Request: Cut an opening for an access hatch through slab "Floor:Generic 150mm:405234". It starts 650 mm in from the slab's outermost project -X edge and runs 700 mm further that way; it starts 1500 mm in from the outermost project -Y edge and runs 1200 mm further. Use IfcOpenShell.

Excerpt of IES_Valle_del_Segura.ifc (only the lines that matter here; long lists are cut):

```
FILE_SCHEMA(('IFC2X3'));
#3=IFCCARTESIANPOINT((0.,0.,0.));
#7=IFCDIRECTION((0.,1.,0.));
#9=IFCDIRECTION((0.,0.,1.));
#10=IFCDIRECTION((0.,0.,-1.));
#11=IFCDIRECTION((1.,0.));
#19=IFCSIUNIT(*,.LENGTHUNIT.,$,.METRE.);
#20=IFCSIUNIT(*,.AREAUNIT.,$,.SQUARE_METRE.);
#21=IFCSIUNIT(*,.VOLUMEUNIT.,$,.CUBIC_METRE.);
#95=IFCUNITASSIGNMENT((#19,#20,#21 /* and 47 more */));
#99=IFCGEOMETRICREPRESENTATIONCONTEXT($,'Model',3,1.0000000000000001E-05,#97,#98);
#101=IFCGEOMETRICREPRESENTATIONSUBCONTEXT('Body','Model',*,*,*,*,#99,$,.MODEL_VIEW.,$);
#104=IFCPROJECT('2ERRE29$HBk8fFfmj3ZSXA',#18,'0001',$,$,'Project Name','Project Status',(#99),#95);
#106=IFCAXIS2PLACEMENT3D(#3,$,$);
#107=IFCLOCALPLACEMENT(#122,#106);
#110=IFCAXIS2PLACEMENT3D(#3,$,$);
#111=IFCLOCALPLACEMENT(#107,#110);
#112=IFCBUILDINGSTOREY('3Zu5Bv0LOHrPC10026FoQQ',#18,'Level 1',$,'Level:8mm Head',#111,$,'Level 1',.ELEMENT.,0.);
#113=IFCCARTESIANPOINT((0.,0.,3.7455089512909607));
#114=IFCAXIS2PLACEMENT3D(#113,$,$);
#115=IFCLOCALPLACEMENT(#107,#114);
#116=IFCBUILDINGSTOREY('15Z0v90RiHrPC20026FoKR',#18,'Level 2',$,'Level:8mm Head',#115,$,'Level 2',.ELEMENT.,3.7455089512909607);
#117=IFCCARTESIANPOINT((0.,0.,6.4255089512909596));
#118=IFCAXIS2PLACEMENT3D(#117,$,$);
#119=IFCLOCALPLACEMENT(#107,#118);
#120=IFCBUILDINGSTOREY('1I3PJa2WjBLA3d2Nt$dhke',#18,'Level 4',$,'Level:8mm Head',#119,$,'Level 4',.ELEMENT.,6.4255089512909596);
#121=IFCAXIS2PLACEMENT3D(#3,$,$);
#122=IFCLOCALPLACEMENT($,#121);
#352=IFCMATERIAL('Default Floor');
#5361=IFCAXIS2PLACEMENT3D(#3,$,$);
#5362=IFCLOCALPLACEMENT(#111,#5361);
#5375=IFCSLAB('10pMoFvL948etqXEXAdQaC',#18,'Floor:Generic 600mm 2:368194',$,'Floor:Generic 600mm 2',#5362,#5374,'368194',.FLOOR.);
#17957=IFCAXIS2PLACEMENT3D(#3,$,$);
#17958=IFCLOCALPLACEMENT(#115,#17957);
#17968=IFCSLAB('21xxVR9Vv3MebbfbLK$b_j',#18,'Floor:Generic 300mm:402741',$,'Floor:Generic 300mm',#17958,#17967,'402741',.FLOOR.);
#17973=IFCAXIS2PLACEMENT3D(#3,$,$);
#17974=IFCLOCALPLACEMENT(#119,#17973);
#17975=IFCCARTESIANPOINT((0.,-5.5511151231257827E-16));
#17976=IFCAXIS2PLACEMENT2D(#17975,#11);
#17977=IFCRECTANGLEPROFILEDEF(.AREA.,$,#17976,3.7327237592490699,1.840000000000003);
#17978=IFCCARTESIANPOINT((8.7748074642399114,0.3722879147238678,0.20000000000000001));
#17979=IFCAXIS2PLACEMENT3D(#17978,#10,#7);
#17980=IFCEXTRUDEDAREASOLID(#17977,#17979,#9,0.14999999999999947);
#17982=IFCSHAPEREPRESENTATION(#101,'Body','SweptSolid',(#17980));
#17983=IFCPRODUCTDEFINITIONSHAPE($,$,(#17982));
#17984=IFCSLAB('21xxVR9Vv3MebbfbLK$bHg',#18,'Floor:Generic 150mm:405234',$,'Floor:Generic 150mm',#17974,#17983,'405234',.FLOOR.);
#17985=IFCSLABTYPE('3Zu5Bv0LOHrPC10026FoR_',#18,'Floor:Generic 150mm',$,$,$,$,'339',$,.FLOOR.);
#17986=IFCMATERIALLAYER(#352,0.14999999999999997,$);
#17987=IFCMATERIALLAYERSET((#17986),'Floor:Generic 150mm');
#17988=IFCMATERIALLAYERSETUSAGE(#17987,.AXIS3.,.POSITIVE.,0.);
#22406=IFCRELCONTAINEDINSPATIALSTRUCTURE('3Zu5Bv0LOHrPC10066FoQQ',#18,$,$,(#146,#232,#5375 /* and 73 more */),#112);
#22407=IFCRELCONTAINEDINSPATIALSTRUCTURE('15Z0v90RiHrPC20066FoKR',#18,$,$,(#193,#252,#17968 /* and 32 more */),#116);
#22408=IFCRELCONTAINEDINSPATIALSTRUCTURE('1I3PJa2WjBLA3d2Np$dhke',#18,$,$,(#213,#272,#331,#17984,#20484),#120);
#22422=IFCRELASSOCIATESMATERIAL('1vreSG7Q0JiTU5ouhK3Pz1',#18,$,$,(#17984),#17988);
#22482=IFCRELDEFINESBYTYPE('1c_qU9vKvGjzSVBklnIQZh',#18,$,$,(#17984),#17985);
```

```python
import numpy as np
import ifcopenshell
import ifcopenshell.api.feature
import ifcopenshell.api.geometry
import ifcopenshell.api.root
import ifcopenshell.geom
import ifcopenshell.util.placement
import ifcopenshell.util.representation
import ifcopenshell.util.shape
import ifcopenshell.util.unit

model = ifcopenshell.open("IES_Valle_del_Segura.ifc")
unit_scale = ifcopenshell.util.unit.calculate_unit_scale(model)
settings = ifcopenshell.geom.settings()


def volume(element):
    """Net volume in cubic metres, openings subtracted."""
    shape = ifcopenshell.geom.create_shape(settings, element)
    return ifcopenshell.util.shape.get_volume(shape.geometry)


slab = model.by_guid("21xxVR9Vv3MebbfbLK$bHg")
before = volume(slab)

# Extent in the slab's own axes, in metres. The edges named are its -X and -Y sides.
slab_shape = ifcopenshell.geom.create_shape(settings, slab)
vertices = ifcopenshell.util.shape.get_vertices(slab_shape.geometry)
x_min, y_min, bottom = vertices.min(axis=0)
top = vertices[:, 2].max()

opening = ifcopenshell.api.root.create_entity(model, ifc_class="IfcOpeningElement", name="Access hatch opening")
context = ifcopenshell.util.representation.get_context(model, "Model", "Body", "MODEL_VIEW")
width, depth = 0.7, 1.2
outline = [(0.0, 0.0), (width, 0.0), (width, depth), (0.0, depth), (0.0, 0.0)]
# Overshoot both faces by 50 mm so the cut is clean.
shape = ifcopenshell.api.geometry.add_slab_representation(
    model, context=context, depth=top - bottom + 0.1, polyline=outline
)
ifcopenshell.api.geometry.assign_representation(model, product=opening, representation=shape)

matrix = ifcopenshell.util.placement.get_local_placement(slab.ObjectPlacement)
matrix[:, 3] = matrix @ np.append(np.array([x_min + 0.65, y_min + 1.5, bottom - 0.05]) / unit_scale, 1.0)
ifcopenshell.api.geometry.edit_object_placement(model, product=opening, matrix=matrix, is_si=False)
ifcopenshell.api.feature.add_feature(model, feature=opening, element=slab)

after = volume(slab)

print(f"slab volume {before:.3f} -> {after:.3f} m3")

model.write("IES_Valle_del_Segura_edited.ifc")
```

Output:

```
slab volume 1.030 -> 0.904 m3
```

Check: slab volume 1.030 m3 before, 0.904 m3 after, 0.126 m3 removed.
